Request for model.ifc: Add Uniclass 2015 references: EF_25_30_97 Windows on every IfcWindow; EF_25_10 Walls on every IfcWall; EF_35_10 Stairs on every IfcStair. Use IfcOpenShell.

First a look at what the model holds.

```python
import ifcopenshell

model = ifcopenshell.open("model.ifc")
print(model.schema)
print("classifications:", [c.Name for c in model.by_type("IfcClassification")])
for ifc_class in ("IfcDoor", "IfcRoof", "IfcStair", "IfcWall", "IfcWindow"):
    print(ifc_class, len(model.by_type(ifc_class)))
```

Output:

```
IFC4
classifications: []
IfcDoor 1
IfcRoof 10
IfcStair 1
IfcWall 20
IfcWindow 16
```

```python
import ifcopenshell
import ifcopenshell.api.classification

model = ifcopenshell.open("model.ifc")

system = ifcopenshell.api.classification.add_classification(model, classification="Uniclass 2015")

codes = {
    "IfcWindow": ("EF_25_30_97", "Windows"),
    "IfcWall": ("EF_25_10", "Walls"),
    "IfcStair": ("EF_35_10", "Stairs"),
}
for ifc_class, (code, name) in codes.items():
    products = model.by_type(ifc_class)
    ifcopenshell.api.classification.add_reference(
        model, products=products, classification=system, identification=code, name=name
    )
    print(code, len(products))

model.write("model_edited.ifc")
```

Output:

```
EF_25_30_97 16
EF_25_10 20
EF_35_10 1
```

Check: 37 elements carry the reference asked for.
